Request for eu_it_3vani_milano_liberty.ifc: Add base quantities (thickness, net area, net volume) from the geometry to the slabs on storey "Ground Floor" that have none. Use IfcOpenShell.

First a look at what the model holds.

```python
import ifcopenshell
import ifcopenshell.util.element
import ifcopenshell.util.unit

model = ifcopenshell.open("eu_it_3vani_milano_liberty.ifc")
print(model.schema)
for unit_type in ("LENGTHUNIT", "AREAUNIT", "VOLUMEUNIT"):
    print(unit_type, ifcopenshell.util.unit.calculate_unit_scale(model, unit_type))
storey = next(s for s in model.by_type("IfcBuildingStorey") if s.Name == "Ground Floor")
slabs = [e for e in ifcopenshell.util.element.get_decomposition(storey) if e.is_a("IfcSlab")]
for e in sorted(slabs, key=lambda e: e.id()):
    print(e.id(), e.is_a(), e.Name, list(ifcopenshell.util.element.get_psets(e, qtos_only=True)), sep=" | ")
```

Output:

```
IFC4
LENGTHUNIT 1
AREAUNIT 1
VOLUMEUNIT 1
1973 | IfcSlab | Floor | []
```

```python
import ifcopenshell
import ifcopenshell.api.pset
import ifcopenshell.geom
import ifcopenshell.util.element
import ifcopenshell.util.shape
import ifcopenshell.util.unit

model = ifcopenshell.open("eu_it_3vani_milano_liberty.ifc")
unit_scale = ifcopenshell.util.unit.calculate_unit_scale(model)
area_scale = ifcopenshell.util.unit.calculate_unit_scale(model, "AREAUNIT")
volume_scale = ifcopenshell.util.unit.calculate_unit_scale(model, "VOLUMEUNIT")
settings = ifcopenshell.geom.settings()

storey = next(s for s in model.by_type("IfcBuildingStorey") if s.Name == "Ground Floor")
slabs = [e for e in ifcopenshell.util.element.get_decomposition(storey) if e.is_a("IfcSlab")]

for e in sorted(slabs, key=lambda e: e.id()):
    if ifcopenshell.util.element.get_psets(e, qtos_only=True, should_inherit=False):
        continue
    # Geometry comes back in metres, in the element's own axes.
    shape = ifcopenshell.geom.create_shape(settings, e)
    values = {
        "Width": ifcopenshell.util.shape.get_z(shape.geometry) / unit_scale,
        "NetArea": ifcopenshell.util.shape.get_footprint_area(shape.geometry) / area_scale,
        "NetVolume": ifcopenshell.util.shape.get_volume(shape.geometry) / volume_scale,
    }
    qto = ifcopenshell.api.pset.add_qto(model, product=e, name="Qto_SlabBaseQuantities")
    ifcopenshell.api.pset.edit_qto(model, qto=qto, properties=values)
    print(e.id(), {k: round(v, 3) for k, v in values.items()})

model.write("eu_it_3vani_milano_liberty_edited.ifc")
```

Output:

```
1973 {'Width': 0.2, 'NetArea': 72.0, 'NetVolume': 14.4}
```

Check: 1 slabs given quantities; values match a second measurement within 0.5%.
